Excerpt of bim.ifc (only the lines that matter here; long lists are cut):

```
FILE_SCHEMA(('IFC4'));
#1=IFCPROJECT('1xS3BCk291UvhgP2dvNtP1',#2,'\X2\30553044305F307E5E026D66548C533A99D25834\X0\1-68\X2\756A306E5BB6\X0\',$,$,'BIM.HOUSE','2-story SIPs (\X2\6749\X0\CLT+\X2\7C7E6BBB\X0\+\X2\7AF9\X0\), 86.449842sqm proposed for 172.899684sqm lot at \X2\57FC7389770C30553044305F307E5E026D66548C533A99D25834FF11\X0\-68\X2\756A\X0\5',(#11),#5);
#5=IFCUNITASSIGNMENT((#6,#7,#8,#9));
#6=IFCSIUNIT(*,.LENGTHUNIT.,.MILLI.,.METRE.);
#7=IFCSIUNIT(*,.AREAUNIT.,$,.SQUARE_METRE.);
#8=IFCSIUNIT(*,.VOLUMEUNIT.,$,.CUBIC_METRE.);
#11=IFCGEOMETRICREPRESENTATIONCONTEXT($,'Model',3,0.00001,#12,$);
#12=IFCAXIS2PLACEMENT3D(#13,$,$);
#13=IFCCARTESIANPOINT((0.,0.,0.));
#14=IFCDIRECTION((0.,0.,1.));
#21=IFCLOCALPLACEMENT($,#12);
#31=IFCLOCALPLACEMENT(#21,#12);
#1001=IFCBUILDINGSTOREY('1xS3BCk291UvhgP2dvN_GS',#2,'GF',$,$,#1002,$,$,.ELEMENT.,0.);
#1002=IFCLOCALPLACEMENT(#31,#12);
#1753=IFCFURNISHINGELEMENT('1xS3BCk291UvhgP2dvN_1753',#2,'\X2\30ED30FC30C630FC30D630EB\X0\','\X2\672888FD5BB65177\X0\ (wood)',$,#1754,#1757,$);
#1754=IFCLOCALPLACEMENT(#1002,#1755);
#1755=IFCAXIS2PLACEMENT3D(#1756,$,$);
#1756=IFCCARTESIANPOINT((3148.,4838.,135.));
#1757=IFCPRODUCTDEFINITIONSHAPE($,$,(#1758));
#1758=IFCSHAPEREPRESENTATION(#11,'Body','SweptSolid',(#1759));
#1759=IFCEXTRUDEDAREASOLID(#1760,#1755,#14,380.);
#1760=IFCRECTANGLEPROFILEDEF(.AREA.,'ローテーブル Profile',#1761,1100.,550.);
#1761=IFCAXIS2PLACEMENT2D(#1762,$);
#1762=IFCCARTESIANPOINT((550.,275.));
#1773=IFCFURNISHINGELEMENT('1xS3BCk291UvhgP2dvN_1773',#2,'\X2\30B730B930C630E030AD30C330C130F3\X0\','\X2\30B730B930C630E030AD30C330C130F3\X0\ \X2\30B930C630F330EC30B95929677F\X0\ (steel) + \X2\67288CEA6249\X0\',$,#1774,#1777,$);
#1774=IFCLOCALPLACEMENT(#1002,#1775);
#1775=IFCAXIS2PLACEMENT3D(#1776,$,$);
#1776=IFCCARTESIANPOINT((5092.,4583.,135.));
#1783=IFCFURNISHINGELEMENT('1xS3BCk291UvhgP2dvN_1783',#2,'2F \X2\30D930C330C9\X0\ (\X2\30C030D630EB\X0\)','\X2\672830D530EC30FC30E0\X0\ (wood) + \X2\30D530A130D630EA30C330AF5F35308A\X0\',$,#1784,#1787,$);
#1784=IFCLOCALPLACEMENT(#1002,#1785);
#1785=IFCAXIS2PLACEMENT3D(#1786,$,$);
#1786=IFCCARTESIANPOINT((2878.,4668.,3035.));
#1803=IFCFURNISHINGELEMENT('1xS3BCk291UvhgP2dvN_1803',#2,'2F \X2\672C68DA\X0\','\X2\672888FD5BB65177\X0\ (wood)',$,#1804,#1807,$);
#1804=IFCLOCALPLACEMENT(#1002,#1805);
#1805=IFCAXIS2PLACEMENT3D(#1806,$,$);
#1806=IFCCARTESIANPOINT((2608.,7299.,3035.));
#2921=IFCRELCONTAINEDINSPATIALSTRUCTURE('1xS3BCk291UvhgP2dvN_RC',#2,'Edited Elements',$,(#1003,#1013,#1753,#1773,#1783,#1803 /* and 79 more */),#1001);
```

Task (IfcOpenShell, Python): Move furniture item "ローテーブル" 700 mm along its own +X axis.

```python
import ifcopenshell
import ifcopenshell.api.geometry
import ifcopenshell.util.placement
import ifcopenshell.util.unit

model = ifcopenshell.open("bim.ifc")
unit_scale = ifcopenshell.util.unit.calculate_unit_scale(model)

item = model.by_guid("1xS3BCk291UvhgP2dvN_1753")
matrix = ifcopenshell.util.placement.get_local_placement(item.ObjectPlacement)
matrix[:3, 3] += matrix[:3, 0] * 0.7 / unit_scale
ifcopenshell.api.geometry.edit_object_placement(model, product=item, matrix=matrix, is_si=False)

print(ifcopenshell.util.placement.get_local_placement(item.ObjectPlacement).round(3) + 0.0)

model.write("bim_updated.ifc")
```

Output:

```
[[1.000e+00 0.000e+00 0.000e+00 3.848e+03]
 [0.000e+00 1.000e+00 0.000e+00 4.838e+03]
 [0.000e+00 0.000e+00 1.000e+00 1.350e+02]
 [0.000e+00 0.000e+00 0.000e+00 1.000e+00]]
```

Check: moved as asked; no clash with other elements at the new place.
